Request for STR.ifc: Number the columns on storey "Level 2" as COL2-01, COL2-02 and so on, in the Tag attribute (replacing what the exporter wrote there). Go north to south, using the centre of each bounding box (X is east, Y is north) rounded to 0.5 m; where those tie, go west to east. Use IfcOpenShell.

First a look at what the model holds.

```python
import ifcopenshell
import ifcopenshell.util.element
import ifcopenshell.util.placement

model = ifcopenshell.open("STR.ifc")
print(model.schema)
storey = next(s for s in model.by_type("IfcBuildingStorey") if s.Name == "Level 2")
columns = [e for e in ifcopenshell.util.element.get_decomposition(storey) if e.is_a("IfcColumn")]
for e in sorted(columns, key=lambda e: e.id()):
    origin = ifcopenshell.util.placement.get_local_placement(e.ObjectPlacement)[:3, 3]
    print(e.id(), e.Tag, e.Name, origin.round(2) + 0.0, sep=" | ")
```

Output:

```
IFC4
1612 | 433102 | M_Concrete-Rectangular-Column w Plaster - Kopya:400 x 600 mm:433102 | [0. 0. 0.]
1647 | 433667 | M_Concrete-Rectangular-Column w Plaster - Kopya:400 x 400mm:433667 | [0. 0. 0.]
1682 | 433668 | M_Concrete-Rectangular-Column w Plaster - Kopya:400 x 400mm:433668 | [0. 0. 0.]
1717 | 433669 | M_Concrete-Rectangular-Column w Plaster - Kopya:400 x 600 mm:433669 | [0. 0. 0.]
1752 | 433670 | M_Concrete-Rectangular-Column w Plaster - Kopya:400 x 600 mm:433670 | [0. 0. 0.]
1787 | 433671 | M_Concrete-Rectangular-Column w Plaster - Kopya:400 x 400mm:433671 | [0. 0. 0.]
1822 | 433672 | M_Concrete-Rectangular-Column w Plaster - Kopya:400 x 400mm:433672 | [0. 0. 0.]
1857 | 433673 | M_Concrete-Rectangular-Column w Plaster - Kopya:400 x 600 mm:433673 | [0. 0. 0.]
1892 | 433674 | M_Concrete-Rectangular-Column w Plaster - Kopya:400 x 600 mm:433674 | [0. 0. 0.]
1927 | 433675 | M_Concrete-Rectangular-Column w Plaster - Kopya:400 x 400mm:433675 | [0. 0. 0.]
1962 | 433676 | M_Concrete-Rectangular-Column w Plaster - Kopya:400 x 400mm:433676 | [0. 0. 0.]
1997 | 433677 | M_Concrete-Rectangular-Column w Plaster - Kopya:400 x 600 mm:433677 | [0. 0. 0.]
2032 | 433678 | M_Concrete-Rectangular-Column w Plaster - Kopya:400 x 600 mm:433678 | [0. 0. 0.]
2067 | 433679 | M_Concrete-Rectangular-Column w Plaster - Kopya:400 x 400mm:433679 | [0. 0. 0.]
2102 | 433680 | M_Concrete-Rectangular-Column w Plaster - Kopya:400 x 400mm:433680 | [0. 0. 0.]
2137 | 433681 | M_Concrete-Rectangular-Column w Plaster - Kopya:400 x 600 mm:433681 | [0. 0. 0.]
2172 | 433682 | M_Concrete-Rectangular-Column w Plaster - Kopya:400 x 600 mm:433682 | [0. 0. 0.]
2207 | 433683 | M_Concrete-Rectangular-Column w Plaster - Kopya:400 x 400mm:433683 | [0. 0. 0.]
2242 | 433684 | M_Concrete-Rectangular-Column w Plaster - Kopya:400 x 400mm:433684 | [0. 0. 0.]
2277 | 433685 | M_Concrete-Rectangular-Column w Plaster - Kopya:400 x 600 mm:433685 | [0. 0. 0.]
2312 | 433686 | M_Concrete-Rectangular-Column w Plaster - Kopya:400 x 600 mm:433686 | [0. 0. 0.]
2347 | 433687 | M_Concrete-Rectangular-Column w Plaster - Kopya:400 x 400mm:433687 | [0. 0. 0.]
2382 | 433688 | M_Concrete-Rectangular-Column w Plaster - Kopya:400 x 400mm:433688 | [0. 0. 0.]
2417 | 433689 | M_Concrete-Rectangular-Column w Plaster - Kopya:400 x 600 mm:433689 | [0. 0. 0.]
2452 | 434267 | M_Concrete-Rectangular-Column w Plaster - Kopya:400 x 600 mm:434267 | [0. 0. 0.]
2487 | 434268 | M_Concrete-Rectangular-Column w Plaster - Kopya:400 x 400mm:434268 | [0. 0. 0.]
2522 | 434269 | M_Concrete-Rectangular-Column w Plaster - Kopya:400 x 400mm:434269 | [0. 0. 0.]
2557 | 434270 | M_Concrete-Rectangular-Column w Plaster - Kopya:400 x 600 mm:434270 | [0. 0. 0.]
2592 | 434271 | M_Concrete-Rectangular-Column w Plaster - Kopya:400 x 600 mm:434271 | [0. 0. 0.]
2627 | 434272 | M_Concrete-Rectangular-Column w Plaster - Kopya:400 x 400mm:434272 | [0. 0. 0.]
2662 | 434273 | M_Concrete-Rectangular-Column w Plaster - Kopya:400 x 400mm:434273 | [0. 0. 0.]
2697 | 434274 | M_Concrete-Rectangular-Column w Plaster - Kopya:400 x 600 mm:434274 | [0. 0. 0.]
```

```python
import ifcopenshell
import ifcopenshell.geom
import ifcopenshell.util.element
import ifcopenshell.util.shape

model = ifcopenshell.open("STR.ifc")
settings = ifcopenshell.geom.settings()
settings.set("use-world-coords", True)


def centre(element):
    shape = ifcopenshell.geom.create_shape(settings, element)
    return ifcopenshell.util.shape.get_bbox_centroid(shape.geometry)


storey = next(s for s in model.by_type("IfcBuildingStorey") if s.Name == "Level 2")
columns = [e for e in ifcopenshell.util.element.get_decomposition(storey) if e.is_a("IfcColumn")]

# Insertion points can sit at a corner or the storey origin, so sort by the geometry (in metres).
centres = {e: centre(e) for e in columns}
columns.sort(key=lambda e: (-round(centres[e][1] / 0.5), centres[e][0]))

for i, e in enumerate(columns, start=1):
    number = f"COL2-{i:02d}"
    e.Tag = number
    print(e.id(), number)

model.write("STR_edited.ifc")
```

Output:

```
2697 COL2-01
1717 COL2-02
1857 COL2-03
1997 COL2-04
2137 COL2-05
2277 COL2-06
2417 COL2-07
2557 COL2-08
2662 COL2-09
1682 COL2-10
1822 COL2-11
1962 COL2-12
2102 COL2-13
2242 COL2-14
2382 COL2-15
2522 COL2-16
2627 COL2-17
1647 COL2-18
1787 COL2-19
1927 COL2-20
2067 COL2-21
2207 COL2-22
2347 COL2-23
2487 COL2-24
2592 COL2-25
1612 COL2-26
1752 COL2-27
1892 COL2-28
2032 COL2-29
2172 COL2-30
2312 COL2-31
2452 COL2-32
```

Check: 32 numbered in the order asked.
